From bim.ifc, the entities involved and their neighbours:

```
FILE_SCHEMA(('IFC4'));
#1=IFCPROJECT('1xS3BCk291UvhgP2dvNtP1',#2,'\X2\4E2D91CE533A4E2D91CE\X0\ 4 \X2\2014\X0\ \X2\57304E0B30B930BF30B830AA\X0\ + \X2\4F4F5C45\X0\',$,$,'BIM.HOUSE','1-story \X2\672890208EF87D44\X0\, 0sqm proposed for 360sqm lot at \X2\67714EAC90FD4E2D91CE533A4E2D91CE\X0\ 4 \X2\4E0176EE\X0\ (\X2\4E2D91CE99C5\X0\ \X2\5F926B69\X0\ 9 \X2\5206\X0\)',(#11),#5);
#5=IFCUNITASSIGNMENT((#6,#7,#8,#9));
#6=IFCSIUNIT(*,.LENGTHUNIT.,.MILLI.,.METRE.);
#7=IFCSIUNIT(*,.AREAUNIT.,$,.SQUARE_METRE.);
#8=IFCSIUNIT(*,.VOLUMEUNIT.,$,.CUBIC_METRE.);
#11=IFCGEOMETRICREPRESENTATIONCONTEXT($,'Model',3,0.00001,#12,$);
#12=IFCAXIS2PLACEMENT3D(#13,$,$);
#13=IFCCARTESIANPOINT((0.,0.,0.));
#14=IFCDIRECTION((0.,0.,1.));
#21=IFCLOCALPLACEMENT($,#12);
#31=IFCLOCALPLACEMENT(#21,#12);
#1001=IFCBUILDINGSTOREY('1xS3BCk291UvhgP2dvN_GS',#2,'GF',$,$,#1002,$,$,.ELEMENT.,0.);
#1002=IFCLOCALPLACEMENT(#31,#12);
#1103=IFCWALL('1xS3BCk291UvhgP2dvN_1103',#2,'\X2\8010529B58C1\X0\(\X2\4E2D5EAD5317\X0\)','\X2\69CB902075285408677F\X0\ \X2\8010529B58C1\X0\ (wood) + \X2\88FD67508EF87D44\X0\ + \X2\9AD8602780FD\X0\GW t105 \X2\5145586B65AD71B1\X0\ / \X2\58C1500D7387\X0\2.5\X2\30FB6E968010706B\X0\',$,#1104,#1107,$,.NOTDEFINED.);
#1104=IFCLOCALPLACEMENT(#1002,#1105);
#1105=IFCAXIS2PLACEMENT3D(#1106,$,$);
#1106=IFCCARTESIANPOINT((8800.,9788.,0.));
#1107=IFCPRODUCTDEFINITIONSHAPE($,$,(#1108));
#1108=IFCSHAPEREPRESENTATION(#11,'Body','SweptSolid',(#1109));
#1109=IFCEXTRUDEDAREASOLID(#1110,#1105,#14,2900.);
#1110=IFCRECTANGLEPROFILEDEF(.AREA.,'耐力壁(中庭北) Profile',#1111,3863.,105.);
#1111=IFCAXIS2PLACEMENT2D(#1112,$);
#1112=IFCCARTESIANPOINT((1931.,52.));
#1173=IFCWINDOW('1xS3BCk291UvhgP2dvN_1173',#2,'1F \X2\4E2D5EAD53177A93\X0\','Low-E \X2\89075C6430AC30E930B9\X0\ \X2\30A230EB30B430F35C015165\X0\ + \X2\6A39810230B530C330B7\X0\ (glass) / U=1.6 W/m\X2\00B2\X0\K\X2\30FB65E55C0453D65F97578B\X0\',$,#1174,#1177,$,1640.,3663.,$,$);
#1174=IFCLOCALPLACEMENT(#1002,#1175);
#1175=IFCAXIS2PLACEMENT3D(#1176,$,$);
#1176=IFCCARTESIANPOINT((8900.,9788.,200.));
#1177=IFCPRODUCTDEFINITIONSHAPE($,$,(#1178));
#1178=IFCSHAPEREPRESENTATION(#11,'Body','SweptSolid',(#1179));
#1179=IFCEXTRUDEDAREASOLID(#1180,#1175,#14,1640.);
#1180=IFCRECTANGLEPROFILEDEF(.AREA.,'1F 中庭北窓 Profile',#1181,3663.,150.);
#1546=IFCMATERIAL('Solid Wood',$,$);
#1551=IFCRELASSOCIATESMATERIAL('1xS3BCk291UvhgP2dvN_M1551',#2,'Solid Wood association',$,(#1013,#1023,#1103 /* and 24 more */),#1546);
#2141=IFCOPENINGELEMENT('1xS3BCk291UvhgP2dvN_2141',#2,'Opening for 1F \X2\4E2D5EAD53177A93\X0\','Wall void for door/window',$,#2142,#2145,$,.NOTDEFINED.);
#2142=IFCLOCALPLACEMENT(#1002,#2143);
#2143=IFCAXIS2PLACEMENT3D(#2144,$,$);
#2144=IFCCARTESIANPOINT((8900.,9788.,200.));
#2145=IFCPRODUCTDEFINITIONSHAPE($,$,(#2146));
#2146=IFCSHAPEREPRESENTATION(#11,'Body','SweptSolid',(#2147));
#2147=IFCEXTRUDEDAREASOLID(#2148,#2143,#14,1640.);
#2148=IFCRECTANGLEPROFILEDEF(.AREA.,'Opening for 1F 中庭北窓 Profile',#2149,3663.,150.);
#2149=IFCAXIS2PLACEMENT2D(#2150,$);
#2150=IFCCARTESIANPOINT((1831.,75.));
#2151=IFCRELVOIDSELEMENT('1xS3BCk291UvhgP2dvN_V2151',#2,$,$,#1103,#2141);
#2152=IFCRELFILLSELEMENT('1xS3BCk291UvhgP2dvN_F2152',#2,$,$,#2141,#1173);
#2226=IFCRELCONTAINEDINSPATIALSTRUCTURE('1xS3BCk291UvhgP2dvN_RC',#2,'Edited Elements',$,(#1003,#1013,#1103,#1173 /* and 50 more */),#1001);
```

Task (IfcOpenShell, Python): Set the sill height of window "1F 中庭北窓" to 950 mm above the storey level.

```python
import numpy as np
import ifcopenshell
import ifcopenshell.api.geometry
import ifcopenshell.geom
import ifcopenshell.util.element
import ifcopenshell.util.placement
import ifcopenshell.util.shape
import ifcopenshell.util.unit

model = ifcopenshell.open("bim.ifc")
unit_scale = ifcopenshell.util.unit.calculate_unit_scale(model)

window = model.by_guid("1xS3BCk291UvhgP2dvN_1173")
opening = window.FillsVoids[0].RelatingOpeningElement
storey = ifcopenshell.util.element.get_container(window, ifc_class="IfcBuildingStorey")
level = ifcopenshell.util.placement.get_local_placement(storey.ObjectPlacement)[2, 3]

# The opening's origin need not be at the sill, so measure its lowest point.
shape = ifcopenshell.geom.create_shape(ifcopenshell.geom.settings(), opening)
bottom = ifcopenshell.util.shape.get_shape_bottom_elevation(shape, shape.geometry) / unit_scale
dz = level + 0.95 / unit_scale - bottom

shift = np.array([0.0, 0.0, dz])
# The window is not placed relative to its opening, so move both.
for product in (opening, window):
    matrix = ifcopenshell.util.placement.get_local_placement(product.ObjectPlacement)
    matrix[:3, 3] += shift
    ifcopenshell.api.geometry.edit_object_placement(model, product=product, matrix=matrix, is_si=False)

print(f"moved by {dz * unit_scale:+.3f} m")

model.write("bim_updated.ifc")
```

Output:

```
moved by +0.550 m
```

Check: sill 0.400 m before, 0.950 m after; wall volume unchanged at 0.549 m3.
